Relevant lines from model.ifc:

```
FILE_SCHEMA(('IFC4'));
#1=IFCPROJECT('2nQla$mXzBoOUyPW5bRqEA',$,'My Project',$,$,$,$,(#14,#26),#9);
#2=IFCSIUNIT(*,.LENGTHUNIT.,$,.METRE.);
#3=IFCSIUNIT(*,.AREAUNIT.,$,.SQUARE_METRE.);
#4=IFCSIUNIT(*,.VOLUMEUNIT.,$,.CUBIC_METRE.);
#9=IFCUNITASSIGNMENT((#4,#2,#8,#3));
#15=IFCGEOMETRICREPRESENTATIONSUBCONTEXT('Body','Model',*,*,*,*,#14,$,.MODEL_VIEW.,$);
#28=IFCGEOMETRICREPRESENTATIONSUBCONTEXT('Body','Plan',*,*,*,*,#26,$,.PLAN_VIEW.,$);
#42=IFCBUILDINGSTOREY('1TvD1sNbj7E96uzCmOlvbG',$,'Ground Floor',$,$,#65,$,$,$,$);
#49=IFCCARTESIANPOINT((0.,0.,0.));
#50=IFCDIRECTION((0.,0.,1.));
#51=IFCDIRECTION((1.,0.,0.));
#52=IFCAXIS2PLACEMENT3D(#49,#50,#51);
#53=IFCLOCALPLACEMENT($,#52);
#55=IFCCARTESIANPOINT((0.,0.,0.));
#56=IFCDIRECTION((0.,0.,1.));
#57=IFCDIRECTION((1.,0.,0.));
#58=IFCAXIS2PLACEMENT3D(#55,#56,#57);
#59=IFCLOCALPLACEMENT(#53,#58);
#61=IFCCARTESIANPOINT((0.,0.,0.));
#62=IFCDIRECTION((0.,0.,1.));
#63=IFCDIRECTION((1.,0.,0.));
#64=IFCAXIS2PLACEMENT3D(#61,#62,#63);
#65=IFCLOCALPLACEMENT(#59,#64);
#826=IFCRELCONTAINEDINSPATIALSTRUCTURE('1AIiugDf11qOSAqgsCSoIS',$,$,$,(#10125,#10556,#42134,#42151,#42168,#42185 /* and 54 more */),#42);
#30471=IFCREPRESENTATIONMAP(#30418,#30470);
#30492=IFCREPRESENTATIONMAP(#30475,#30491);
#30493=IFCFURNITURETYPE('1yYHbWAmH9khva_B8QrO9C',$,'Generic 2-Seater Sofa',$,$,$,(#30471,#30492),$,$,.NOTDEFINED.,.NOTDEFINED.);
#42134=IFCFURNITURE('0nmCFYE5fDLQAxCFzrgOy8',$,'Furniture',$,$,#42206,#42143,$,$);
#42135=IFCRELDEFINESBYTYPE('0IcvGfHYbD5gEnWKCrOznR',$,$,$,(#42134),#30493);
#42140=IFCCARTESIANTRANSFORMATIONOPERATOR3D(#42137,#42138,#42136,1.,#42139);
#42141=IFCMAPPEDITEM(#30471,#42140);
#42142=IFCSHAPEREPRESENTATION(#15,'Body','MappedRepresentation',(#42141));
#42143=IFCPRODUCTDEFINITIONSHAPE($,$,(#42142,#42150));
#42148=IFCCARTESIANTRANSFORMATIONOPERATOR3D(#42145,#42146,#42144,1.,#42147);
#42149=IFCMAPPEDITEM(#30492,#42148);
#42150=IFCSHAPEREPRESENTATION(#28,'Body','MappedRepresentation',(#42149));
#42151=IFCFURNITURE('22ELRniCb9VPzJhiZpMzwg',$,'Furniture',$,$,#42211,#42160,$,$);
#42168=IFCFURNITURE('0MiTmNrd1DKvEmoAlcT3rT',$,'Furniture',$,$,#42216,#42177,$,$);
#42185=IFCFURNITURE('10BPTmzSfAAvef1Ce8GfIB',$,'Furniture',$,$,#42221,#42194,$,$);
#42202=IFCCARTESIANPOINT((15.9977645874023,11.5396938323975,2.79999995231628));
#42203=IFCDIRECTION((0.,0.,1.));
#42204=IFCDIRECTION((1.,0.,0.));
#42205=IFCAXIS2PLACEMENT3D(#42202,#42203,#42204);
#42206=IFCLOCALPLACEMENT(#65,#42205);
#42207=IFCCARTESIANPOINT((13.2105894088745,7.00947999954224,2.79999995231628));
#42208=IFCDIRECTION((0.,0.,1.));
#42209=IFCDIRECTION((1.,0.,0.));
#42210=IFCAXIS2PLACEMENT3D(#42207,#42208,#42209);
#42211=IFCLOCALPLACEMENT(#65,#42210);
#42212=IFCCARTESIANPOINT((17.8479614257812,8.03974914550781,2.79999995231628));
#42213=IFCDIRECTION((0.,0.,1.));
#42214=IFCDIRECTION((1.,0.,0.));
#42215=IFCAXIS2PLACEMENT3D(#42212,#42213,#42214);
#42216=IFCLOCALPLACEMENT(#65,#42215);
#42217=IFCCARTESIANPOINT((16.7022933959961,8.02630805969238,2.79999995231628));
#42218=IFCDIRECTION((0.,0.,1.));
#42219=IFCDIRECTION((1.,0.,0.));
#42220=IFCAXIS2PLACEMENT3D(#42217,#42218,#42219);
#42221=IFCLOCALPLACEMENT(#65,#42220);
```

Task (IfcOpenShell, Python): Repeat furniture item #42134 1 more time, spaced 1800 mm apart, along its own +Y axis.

```python
import ifcopenshell
import ifcopenshell.api.geometry
import ifcopenshell.api.root
import ifcopenshell.util.element
import ifcopenshell.util.placement
import ifcopenshell.util.unit

model = ifcopenshell.open("model.ifc")
unit_scale = ifcopenshell.util.unit.calculate_unit_scale(model)

source = model.by_guid("0nmCFYE5fDLQAxCFzrgOy8")
base = ifcopenshell.util.placement.get_local_placement(source.ObjectPlacement)
step = base[:3, 1] * 1.8 / unit_scale

for i in range(1, 2):
    copy = ifcopenshell.api.root.copy_class(model, product=source)
    copy.Representation = ifcopenshell.util.element.copy_deep(
        model, source.Representation, exclude=["IfcGeometricRepresentationContext", "IfcRepresentationMap"]
    )
    matrix = base.copy()
    matrix[:3, 3] += i * step
    print("added at", matrix[:3, 3].round(3) + 0.0)
    ifcopenshell.api.geometry.edit_object_placement(model, product=copy, matrix=matrix, is_si=False)

model.write("model-out.ifc")
```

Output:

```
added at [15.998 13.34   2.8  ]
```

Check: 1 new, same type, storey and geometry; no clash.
